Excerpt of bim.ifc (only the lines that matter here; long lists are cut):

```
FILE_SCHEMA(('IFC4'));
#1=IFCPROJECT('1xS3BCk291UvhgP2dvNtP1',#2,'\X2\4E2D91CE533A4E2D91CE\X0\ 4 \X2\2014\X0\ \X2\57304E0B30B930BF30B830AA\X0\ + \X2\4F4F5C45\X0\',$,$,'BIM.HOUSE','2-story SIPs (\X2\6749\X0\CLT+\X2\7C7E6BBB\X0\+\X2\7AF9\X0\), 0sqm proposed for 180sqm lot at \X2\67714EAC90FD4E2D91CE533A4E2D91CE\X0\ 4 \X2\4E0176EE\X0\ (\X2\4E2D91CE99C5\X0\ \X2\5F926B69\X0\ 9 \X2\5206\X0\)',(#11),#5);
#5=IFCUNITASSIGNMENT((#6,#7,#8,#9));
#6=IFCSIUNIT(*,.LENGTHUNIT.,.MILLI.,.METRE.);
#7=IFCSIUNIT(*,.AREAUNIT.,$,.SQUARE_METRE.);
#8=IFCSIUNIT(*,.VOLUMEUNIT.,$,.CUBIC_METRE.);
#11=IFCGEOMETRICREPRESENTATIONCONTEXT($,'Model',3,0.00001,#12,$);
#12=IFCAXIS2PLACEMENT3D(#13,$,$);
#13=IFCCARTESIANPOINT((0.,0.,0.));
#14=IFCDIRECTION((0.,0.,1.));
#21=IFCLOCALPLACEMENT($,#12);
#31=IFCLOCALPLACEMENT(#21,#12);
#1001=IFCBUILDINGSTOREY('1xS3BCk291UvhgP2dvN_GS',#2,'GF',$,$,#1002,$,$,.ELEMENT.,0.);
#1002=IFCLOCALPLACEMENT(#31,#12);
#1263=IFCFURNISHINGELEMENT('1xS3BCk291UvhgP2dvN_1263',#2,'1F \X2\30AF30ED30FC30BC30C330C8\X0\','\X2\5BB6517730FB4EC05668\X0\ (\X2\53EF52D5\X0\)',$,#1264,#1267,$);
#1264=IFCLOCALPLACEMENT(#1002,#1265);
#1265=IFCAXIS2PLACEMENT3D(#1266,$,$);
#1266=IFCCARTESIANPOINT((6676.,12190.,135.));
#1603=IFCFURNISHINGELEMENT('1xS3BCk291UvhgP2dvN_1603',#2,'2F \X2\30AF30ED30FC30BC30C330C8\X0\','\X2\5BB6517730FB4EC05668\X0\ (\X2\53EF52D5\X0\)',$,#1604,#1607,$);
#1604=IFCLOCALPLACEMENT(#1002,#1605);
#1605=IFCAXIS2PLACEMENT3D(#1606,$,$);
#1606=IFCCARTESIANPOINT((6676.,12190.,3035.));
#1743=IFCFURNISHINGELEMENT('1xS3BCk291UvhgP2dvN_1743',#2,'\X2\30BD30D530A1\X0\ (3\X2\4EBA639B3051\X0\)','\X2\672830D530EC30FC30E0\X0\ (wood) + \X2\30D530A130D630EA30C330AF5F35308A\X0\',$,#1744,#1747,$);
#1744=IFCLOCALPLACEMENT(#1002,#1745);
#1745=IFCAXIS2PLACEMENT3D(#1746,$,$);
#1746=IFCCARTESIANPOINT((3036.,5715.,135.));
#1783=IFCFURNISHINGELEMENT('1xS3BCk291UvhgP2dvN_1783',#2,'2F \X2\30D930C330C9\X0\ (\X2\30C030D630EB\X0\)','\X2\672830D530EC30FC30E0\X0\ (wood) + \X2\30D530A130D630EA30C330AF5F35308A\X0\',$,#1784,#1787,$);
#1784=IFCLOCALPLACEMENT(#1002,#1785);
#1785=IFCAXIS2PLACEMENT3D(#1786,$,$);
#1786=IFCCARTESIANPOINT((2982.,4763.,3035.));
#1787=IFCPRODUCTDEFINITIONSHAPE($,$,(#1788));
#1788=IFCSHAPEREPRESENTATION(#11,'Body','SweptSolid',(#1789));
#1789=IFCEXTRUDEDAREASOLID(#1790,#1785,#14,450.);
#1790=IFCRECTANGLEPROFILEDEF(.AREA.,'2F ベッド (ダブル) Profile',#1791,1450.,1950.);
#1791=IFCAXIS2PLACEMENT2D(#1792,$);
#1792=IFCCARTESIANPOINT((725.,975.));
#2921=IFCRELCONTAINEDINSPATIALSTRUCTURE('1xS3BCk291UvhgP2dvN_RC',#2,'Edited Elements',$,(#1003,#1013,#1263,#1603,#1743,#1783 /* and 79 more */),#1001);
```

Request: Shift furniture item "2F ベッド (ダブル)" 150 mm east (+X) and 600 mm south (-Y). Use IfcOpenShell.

```python
import ifcopenshell
import ifcopenshell.api.geometry
import ifcopenshell.util.placement
import ifcopenshell.util.unit

model = ifcopenshell.open("bim.ifc")
unit_scale = ifcopenshell.util.unit.calculate_unit_scale(model)

item = model.by_guid("1xS3BCk291UvhgP2dvN_1783")
matrix = ifcopenshell.util.placement.get_local_placement(item.ObjectPlacement)
matrix[0, 3] += 0.15 / unit_scale
matrix[1, 3] -= 0.6 / unit_scale
ifcopenshell.api.geometry.edit_object_placement(model, product=item, matrix=matrix, is_si=False)

print(ifcopenshell.util.placement.get_local_placement(item.ObjectPlacement).round(3) + 0.0)

model.write("bim_rev.ifc")
```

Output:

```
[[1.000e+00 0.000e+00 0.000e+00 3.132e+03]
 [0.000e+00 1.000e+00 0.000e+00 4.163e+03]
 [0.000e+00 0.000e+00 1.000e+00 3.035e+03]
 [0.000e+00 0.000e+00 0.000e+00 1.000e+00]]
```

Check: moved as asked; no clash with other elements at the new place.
